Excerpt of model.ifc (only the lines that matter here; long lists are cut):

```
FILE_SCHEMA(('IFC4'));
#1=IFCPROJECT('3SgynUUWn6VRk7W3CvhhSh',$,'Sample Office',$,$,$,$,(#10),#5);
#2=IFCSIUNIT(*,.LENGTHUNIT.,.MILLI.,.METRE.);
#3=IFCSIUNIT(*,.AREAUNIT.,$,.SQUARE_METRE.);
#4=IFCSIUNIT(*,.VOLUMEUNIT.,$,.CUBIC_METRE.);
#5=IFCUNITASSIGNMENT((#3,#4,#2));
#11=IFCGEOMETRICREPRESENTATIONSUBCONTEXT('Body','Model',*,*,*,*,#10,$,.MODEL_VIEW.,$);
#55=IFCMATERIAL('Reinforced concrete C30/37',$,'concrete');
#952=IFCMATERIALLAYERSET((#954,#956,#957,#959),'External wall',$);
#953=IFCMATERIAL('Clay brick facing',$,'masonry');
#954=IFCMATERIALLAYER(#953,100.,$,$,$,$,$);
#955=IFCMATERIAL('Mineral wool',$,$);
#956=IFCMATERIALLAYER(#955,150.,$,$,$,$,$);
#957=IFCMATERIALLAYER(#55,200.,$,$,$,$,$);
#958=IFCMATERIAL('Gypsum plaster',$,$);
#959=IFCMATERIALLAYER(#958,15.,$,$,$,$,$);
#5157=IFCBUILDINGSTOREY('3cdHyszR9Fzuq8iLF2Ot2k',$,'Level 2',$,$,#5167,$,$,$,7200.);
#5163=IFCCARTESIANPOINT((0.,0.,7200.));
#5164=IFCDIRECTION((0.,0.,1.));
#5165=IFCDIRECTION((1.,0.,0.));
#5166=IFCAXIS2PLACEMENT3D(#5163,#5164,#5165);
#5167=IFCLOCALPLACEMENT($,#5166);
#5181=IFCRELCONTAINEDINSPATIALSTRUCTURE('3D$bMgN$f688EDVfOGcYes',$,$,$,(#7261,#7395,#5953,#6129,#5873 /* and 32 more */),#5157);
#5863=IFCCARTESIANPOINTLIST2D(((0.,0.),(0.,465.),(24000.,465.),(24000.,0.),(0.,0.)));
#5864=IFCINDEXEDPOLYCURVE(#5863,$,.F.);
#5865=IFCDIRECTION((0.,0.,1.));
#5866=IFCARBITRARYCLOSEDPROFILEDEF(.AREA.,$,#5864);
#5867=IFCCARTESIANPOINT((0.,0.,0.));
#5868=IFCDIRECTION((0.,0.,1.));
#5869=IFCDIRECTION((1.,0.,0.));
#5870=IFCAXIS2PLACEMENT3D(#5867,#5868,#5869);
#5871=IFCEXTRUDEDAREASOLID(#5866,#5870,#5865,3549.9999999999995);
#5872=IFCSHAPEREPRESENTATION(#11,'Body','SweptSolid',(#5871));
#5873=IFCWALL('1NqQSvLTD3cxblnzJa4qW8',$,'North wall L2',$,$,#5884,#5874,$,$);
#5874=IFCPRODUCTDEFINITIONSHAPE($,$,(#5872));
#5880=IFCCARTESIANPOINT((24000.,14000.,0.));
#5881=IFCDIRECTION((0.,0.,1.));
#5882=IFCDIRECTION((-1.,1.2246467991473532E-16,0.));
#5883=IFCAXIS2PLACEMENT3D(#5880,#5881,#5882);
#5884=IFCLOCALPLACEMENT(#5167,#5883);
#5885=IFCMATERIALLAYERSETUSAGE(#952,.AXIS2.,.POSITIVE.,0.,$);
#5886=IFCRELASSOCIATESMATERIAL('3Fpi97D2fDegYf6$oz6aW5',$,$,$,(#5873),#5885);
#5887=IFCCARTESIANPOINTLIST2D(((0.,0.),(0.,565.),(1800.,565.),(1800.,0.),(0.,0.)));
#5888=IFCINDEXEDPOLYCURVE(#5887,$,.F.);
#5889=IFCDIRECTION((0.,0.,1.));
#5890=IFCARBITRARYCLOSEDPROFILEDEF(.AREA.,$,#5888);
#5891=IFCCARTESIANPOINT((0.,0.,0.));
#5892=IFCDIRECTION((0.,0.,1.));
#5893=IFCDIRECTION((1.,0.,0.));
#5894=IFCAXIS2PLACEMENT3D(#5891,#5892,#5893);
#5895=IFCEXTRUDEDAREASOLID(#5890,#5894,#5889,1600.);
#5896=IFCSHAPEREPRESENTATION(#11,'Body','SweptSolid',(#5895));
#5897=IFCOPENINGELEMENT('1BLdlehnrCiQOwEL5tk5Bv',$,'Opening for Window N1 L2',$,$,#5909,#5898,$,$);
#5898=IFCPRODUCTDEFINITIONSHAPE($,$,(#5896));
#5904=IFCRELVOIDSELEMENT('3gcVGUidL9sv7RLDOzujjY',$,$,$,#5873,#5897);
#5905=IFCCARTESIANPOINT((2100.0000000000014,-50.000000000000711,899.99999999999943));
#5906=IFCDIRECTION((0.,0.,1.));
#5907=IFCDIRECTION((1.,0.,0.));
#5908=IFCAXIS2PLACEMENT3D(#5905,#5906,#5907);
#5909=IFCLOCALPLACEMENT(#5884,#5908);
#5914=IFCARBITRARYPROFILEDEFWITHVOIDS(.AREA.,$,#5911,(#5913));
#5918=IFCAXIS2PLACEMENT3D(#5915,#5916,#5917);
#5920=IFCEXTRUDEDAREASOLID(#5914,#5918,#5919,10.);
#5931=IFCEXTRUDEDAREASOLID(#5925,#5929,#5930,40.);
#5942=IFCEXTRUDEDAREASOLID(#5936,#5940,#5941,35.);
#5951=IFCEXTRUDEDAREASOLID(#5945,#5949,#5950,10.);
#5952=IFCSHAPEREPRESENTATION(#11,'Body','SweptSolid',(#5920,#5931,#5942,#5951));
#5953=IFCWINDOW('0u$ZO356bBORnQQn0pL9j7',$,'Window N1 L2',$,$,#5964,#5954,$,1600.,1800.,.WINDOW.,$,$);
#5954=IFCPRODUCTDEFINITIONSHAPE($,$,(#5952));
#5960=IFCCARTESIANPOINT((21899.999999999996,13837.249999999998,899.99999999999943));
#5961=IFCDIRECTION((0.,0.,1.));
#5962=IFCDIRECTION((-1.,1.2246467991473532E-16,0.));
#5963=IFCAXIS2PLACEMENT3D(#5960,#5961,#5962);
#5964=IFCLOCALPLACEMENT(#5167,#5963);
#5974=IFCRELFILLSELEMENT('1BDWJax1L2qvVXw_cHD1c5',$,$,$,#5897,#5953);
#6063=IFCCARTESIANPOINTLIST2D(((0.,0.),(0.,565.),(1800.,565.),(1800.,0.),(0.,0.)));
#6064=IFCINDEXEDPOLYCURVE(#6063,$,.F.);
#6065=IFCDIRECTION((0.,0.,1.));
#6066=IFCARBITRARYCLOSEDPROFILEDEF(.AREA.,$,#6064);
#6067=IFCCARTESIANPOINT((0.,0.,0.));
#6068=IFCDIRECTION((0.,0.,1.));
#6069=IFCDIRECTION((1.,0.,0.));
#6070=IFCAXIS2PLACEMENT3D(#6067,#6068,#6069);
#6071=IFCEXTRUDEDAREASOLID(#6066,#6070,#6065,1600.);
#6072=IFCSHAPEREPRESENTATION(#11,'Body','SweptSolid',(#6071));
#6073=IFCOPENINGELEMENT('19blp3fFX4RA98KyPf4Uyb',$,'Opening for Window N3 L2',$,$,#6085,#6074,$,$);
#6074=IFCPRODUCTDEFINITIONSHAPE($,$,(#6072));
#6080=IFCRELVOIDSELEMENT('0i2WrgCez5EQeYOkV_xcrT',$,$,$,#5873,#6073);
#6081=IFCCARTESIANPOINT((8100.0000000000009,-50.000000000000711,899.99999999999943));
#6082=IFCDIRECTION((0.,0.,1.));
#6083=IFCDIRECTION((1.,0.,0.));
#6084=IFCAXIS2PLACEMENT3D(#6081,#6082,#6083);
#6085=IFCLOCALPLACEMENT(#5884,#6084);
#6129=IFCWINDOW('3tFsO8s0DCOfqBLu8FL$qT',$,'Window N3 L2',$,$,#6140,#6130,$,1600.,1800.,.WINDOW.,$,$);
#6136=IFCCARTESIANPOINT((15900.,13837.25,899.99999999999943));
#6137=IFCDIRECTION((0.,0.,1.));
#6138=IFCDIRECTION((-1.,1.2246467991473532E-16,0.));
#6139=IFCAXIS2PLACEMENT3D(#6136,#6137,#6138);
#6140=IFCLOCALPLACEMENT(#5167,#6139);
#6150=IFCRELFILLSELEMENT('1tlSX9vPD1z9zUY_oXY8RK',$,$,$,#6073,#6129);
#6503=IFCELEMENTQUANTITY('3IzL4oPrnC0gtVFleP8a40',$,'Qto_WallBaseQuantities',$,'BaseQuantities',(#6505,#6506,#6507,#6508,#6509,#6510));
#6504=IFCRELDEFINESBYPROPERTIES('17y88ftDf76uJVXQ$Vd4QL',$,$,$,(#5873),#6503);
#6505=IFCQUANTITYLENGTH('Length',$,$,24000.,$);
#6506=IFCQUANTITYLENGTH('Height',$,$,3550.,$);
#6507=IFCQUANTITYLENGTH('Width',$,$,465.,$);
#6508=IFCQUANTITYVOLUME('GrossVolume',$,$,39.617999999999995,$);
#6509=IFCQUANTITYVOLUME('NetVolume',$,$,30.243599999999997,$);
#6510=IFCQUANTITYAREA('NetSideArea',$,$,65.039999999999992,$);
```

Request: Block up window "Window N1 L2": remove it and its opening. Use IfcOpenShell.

```python
import ifcopenshell
import ifcopenshell.api.feature
import ifcopenshell.api.pset
import ifcopenshell.api.root
import ifcopenshell.geom
import ifcopenshell.util.element
import ifcopenshell.util.shape
import ifcopenshell.util.unit

model = ifcopenshell.open("model.ifc")
area_scale = ifcopenshell.util.unit.calculate_unit_scale(model, "AREAUNIT")
volume_scale = ifcopenshell.util.unit.calculate_unit_scale(model, "VOLUMEUNIT")
settings = ifcopenshell.geom.settings()


def volume(element):
    """Net volume in cubic metres, openings subtracted."""
    shape = ifcopenshell.geom.create_shape(settings, element)
    return ifcopenshell.util.shape.get_volume(shape.geometry)


window = model.by_guid("0u$ZO356bBORnQQn0pL9j7")
opening = window.FillsVoids[0].RelatingOpeningElement
wall = opening.VoidsElements[0].RelatingBuildingElement
before = volume(wall)

ifcopenshell.api.root.remove_product(model, product=window)
ifcopenshell.api.feature.remove_feature(model, feature=opening)

after = volume(wall)
thickness = 0.465  # wall thickness in metres

# Update the wall's stored quantities.
qto = model.by_id(ifcopenshell.util.element.get_pset(wall, "Qto_WallBaseQuantities", should_inherit=False)["id"])
ifcopenshell.api.pset.edit_qto(model, qto=qto, properties={
    "NetVolume": after / volume_scale,
    "NetSideArea": after / thickness / area_scale,
})

print(f"wall volume {before:.3f} -> {after:.3f} m3")

model.write("model_updated.ifc")
```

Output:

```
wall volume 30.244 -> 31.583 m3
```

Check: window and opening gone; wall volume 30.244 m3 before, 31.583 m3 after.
